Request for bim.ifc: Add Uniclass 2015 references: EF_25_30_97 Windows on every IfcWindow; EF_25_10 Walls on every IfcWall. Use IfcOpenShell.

First a look at what the model holds.

```python
import ifcopenshell

model = ifcopenshell.open("bim.ifc")
print(model.schema)
print("classifications:", [c.Name for c in model.by_type("IfcClassification")])
for ifc_class in ("IfcDoor", "IfcRoof", "IfcStair", "IfcWall", "IfcWindow"):
    print(ifc_class, len(model.by_type(ifc_class)))
```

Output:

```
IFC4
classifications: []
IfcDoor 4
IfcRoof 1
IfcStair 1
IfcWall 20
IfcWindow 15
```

```python
import ifcopenshell
import ifcopenshell.api.classification

model = ifcopenshell.open("bim.ifc")

system = ifcopenshell.api.classification.add_classification(model, classification="Uniclass 2015")

codes = {
    "IfcWindow": ("EF_25_30_97", "Windows"),
    "IfcWall": ("EF_25_10", "Walls"),
}
for ifc_class, (code, name) in codes.items():
    products = model.by_type(ifc_class)
    ifcopenshell.api.classification.add_reference(
        model, products=products, classification=system, identification=code, name=name
    )
    print(code, len(products))

model.write("bim_edited.ifc")
```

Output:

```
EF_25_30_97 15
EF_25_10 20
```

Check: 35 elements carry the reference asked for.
